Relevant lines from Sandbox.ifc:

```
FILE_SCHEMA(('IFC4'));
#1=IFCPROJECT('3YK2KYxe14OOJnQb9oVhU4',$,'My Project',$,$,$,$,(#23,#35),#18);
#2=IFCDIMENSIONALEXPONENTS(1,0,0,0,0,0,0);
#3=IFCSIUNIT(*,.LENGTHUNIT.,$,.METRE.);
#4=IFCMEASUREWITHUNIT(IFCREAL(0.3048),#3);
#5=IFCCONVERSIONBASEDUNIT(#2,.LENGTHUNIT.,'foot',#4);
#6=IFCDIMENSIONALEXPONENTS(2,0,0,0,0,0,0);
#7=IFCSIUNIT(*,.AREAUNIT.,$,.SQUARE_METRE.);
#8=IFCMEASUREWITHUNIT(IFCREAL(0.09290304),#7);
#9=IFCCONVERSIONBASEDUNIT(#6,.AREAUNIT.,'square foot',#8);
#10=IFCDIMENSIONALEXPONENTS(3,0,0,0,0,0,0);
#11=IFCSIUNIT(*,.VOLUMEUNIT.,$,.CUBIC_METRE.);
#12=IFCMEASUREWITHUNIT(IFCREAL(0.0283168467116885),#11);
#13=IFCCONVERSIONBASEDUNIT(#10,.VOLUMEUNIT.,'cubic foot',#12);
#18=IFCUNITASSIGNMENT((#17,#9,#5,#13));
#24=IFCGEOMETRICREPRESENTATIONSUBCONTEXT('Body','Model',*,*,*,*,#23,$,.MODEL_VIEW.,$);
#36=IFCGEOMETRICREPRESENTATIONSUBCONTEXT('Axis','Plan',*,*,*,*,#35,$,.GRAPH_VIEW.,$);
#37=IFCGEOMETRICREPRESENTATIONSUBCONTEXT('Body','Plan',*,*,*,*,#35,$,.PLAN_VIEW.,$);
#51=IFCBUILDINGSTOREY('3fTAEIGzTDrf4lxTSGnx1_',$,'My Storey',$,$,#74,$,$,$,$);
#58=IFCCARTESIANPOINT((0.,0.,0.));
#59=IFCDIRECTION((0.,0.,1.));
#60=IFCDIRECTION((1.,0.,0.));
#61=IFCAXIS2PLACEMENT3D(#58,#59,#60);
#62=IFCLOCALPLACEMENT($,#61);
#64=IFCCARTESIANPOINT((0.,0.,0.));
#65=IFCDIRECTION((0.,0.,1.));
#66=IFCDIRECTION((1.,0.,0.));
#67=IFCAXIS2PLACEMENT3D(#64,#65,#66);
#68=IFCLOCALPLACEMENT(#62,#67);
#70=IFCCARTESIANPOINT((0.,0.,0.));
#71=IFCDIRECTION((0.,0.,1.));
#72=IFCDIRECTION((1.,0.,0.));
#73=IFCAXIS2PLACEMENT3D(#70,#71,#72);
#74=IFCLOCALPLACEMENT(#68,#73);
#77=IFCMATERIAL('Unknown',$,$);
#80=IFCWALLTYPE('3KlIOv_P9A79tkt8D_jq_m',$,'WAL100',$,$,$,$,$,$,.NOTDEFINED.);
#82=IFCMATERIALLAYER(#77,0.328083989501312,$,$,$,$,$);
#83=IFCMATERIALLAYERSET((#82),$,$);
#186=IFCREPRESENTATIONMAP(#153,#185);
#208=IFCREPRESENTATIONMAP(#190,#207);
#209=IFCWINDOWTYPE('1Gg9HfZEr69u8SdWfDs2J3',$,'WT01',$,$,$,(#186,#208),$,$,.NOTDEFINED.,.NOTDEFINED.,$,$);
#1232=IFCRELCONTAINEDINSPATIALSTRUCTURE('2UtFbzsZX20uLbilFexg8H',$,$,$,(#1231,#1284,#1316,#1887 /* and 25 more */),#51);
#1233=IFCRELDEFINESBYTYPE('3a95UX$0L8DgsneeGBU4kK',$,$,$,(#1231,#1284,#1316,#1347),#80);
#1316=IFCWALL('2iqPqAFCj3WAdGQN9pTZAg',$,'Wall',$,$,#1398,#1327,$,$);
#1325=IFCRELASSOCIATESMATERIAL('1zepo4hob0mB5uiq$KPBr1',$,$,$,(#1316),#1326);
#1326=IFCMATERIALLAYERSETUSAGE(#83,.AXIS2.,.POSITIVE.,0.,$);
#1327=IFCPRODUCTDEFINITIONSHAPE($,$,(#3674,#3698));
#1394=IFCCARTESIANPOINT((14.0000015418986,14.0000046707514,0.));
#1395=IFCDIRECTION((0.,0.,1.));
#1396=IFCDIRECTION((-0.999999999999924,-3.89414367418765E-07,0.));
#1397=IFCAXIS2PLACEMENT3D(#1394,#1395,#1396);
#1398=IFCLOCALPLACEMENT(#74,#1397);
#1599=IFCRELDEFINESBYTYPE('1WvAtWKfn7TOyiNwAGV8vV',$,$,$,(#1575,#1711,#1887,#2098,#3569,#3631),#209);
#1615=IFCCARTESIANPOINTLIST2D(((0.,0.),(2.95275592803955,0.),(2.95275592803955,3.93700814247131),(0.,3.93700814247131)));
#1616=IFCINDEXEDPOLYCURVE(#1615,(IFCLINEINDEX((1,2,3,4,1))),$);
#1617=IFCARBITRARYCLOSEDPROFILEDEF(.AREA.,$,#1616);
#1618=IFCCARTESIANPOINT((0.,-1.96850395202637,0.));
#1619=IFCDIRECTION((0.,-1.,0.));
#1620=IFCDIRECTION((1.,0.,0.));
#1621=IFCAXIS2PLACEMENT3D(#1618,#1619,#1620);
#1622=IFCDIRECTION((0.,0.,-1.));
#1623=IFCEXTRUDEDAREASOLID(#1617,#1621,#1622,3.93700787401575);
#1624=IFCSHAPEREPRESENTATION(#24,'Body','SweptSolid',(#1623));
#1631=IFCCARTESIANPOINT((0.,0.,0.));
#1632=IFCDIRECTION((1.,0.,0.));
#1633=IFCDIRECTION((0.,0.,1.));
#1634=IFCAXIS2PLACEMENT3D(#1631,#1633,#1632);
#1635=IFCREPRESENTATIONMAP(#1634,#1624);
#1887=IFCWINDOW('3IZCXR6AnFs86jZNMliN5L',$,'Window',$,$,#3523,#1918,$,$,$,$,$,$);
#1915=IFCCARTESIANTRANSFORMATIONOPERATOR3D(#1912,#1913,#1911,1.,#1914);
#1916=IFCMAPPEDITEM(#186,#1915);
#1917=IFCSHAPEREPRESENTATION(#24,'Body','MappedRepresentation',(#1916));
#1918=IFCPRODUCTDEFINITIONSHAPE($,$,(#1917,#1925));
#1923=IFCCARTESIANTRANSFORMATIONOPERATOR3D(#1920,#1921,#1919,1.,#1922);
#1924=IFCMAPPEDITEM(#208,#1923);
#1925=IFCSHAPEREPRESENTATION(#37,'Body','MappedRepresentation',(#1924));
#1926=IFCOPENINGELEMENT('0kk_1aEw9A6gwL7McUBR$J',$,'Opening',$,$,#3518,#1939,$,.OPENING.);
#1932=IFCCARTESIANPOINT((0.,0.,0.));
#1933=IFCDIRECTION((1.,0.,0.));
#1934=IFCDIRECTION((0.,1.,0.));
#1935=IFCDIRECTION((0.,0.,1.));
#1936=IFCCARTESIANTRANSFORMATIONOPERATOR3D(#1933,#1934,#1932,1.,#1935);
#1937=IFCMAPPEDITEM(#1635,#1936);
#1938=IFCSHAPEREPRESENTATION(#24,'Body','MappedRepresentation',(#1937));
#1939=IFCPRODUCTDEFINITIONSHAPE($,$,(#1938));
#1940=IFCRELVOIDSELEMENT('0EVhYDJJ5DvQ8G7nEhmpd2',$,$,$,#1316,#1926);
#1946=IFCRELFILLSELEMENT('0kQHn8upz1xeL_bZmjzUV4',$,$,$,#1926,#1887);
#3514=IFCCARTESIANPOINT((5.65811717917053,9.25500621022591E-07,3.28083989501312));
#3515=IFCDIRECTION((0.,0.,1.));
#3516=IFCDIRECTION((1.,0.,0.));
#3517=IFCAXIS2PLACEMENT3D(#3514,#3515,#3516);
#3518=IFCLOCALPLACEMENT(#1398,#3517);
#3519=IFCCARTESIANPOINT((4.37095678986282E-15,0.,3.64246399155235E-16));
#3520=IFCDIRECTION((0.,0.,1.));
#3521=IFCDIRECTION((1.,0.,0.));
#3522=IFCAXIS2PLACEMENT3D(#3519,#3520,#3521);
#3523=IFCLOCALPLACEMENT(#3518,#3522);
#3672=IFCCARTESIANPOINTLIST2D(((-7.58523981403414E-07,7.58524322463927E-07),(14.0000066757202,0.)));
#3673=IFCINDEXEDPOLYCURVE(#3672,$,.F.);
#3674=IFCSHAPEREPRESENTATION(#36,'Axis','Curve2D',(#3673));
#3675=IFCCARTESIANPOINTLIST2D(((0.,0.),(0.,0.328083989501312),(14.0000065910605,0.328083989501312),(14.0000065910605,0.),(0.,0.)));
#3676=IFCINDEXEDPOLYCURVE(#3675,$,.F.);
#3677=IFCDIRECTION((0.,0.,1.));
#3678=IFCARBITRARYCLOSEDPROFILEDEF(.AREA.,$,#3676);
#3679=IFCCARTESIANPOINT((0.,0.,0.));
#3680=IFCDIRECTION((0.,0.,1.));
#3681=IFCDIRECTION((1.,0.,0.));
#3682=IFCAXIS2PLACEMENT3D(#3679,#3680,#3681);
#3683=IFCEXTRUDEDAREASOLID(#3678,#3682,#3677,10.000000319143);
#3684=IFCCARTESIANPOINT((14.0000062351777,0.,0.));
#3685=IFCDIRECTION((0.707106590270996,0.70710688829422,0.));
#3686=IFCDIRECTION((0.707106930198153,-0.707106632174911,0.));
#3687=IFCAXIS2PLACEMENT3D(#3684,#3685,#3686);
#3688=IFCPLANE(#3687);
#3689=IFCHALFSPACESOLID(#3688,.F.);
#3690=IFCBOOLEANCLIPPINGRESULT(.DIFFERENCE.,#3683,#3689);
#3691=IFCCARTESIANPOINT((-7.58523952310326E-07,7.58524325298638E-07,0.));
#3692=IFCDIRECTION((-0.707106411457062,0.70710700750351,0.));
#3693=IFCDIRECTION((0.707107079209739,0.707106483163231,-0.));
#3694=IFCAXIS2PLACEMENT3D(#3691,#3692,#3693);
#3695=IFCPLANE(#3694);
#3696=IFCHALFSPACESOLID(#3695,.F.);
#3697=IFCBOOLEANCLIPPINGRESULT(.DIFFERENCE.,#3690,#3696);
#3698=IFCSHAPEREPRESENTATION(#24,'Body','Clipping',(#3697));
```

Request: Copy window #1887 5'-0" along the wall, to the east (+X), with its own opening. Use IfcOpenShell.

```python
import ifcopenshell
import ifcopenshell.api.feature
import ifcopenshell.api.geometry
import ifcopenshell.api.root
import ifcopenshell.geom
import ifcopenshell.util.element
import ifcopenshell.util.placement
import ifcopenshell.util.shape
import ifcopenshell.util.unit

model = ifcopenshell.open("Sandbox.ifc")
unit_scale = ifcopenshell.util.unit.calculate_unit_scale(model)
settings = ifcopenshell.geom.settings()


def volume(element):
    """Net volume in cubic metres, openings subtracted."""
    shape = ifcopenshell.geom.create_shape(settings, element)
    return ifcopenshell.util.shape.get_volume(shape.geometry)


window = model.by_id(1887)
opening = window.FillsVoids[0].RelatingOpeningElement
wall = opening.VoidsElements[0].RelatingBuildingElement
before = volume(wall)
shift = ifcopenshell.util.placement.get_local_placement(wall.ObjectPlacement)[:3, 0] * -60 * 0.0254 / unit_scale

# copy_class copies the void relationship, type, container and properties, but no geometry.
new_opening = ifcopenshell.api.root.copy_class(model, product=opening)
new_opening.Representation = ifcopenshell.util.element.copy_deep(
    model, opening.Representation, exclude=["IfcGeometricRepresentationContext", "IfcRepresentationMap"]
)
new_window = ifcopenshell.api.root.copy_class(model, product=window)
new_window.Representation = ifcopenshell.util.element.copy_deep(
    model, window.Representation, exclude=["IfcGeometricRepresentationContext", "IfcRepresentationMap"]
)
ifcopenshell.api.feature.add_filling(model, opening=new_opening, element=new_window)

for old, new in ((opening, new_opening), (window, new_window)):
    matrix = ifcopenshell.util.placement.get_local_placement(old.ObjectPlacement)
    matrix[:3, 3] += shift
    ifcopenshell.api.geometry.edit_object_placement(model, product=new, matrix=matrix, is_si=False)

after = volume(wall)

print(f"wall volume {before:.3f} -> {after:.3f} m3")

model.write("Sandbox_edited.ifc")
```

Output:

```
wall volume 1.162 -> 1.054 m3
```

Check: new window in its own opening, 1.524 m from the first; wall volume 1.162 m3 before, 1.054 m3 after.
